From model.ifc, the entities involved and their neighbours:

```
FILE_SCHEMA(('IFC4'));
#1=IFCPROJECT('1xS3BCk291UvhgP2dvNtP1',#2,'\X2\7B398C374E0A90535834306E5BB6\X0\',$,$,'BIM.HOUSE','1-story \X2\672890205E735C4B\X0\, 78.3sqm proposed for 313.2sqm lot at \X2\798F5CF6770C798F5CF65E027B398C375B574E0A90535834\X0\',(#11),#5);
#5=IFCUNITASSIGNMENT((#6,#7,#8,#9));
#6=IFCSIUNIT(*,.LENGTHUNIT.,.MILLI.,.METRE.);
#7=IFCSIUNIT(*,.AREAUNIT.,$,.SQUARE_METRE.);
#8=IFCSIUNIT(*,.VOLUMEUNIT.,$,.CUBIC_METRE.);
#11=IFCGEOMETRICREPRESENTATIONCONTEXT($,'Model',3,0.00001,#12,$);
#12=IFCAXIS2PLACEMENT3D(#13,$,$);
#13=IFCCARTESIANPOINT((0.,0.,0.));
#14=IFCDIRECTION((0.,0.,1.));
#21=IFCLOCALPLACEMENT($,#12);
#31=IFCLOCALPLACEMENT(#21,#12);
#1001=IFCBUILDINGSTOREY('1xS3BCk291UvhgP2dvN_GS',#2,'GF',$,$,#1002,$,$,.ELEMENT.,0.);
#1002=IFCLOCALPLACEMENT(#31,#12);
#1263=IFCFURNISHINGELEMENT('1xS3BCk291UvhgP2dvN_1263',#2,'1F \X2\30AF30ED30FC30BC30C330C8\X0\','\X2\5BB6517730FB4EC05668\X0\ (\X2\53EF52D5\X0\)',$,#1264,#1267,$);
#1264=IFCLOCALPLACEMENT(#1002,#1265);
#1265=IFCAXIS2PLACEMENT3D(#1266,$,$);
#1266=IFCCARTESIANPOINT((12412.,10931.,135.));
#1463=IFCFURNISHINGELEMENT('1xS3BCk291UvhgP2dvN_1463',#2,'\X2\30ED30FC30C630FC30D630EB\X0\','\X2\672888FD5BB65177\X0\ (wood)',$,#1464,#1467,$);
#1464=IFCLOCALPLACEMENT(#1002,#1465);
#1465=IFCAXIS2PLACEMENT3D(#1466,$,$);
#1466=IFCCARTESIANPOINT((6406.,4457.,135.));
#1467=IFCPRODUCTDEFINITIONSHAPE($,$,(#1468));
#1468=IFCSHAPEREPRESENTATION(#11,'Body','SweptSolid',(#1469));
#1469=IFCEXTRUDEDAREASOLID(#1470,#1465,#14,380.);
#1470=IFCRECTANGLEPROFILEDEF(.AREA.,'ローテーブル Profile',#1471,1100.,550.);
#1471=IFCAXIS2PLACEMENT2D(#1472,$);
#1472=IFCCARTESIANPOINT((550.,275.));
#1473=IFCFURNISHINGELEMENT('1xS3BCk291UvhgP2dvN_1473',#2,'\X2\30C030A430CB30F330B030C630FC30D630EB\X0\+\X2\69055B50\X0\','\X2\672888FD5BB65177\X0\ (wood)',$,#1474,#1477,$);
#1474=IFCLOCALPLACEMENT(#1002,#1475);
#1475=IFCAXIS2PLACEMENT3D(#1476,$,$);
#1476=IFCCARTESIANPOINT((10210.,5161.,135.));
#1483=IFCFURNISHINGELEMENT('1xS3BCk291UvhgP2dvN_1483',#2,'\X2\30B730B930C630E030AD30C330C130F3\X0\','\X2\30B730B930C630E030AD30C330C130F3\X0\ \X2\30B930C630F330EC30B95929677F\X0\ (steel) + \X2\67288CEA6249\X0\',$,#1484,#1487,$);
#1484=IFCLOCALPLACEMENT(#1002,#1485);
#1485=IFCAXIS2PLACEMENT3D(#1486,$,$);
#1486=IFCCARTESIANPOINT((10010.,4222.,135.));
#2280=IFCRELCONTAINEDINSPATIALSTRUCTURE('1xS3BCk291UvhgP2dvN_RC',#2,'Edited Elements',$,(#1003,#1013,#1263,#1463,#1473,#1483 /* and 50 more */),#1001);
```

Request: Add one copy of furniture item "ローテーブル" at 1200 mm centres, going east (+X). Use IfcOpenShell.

```python
import numpy as np
import ifcopenshell
import ifcopenshell.api.geometry
import ifcopenshell.api.root
import ifcopenshell.util.element
import ifcopenshell.util.placement

model = ifcopenshell.open("model.ifc")


def reuse_history(source, copy):
    """copy_class also copies each property set's owner history, people and application; keep the originals."""
    for rel in copy.IsDefinedBy:
        if rel.is_a("IfcRelDefinesByProperties") and (history := rel.RelatingPropertyDefinition.OwnerHistory):
            rel.RelatingPropertyDefinition.OwnerHistory = source.OwnerHistory
            ifcopenshell.util.element.remove_deep2(model, history)


source = model.by_guid("1xS3BCk291UvhgP2dvN_1463")
base = ifcopenshell.util.placement.get_local_placement(source.ObjectPlacement)
step = np.array([1.0, 0.0, 0.0]) * 1200.0

for i in range(1, 2):
    copy = ifcopenshell.api.root.copy_class(model, product=source)
    copy.Representation = ifcopenshell.util.element.copy_deep(
        model, source.Representation, exclude=["IfcGeometricRepresentationContext", "IfcRepresentationMap"]
    )
    reuse_history(source, copy)
    matrix = base.copy()
    matrix[:3, 3] += i * step
    print("added at", matrix[:3, 3].round(3) + 0.0)
    ifcopenshell.api.geometry.edit_object_placement(model, product=copy, matrix=matrix, is_si=False)

model.write("model_v2.ifc")
```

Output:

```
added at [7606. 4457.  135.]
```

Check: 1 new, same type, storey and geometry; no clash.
